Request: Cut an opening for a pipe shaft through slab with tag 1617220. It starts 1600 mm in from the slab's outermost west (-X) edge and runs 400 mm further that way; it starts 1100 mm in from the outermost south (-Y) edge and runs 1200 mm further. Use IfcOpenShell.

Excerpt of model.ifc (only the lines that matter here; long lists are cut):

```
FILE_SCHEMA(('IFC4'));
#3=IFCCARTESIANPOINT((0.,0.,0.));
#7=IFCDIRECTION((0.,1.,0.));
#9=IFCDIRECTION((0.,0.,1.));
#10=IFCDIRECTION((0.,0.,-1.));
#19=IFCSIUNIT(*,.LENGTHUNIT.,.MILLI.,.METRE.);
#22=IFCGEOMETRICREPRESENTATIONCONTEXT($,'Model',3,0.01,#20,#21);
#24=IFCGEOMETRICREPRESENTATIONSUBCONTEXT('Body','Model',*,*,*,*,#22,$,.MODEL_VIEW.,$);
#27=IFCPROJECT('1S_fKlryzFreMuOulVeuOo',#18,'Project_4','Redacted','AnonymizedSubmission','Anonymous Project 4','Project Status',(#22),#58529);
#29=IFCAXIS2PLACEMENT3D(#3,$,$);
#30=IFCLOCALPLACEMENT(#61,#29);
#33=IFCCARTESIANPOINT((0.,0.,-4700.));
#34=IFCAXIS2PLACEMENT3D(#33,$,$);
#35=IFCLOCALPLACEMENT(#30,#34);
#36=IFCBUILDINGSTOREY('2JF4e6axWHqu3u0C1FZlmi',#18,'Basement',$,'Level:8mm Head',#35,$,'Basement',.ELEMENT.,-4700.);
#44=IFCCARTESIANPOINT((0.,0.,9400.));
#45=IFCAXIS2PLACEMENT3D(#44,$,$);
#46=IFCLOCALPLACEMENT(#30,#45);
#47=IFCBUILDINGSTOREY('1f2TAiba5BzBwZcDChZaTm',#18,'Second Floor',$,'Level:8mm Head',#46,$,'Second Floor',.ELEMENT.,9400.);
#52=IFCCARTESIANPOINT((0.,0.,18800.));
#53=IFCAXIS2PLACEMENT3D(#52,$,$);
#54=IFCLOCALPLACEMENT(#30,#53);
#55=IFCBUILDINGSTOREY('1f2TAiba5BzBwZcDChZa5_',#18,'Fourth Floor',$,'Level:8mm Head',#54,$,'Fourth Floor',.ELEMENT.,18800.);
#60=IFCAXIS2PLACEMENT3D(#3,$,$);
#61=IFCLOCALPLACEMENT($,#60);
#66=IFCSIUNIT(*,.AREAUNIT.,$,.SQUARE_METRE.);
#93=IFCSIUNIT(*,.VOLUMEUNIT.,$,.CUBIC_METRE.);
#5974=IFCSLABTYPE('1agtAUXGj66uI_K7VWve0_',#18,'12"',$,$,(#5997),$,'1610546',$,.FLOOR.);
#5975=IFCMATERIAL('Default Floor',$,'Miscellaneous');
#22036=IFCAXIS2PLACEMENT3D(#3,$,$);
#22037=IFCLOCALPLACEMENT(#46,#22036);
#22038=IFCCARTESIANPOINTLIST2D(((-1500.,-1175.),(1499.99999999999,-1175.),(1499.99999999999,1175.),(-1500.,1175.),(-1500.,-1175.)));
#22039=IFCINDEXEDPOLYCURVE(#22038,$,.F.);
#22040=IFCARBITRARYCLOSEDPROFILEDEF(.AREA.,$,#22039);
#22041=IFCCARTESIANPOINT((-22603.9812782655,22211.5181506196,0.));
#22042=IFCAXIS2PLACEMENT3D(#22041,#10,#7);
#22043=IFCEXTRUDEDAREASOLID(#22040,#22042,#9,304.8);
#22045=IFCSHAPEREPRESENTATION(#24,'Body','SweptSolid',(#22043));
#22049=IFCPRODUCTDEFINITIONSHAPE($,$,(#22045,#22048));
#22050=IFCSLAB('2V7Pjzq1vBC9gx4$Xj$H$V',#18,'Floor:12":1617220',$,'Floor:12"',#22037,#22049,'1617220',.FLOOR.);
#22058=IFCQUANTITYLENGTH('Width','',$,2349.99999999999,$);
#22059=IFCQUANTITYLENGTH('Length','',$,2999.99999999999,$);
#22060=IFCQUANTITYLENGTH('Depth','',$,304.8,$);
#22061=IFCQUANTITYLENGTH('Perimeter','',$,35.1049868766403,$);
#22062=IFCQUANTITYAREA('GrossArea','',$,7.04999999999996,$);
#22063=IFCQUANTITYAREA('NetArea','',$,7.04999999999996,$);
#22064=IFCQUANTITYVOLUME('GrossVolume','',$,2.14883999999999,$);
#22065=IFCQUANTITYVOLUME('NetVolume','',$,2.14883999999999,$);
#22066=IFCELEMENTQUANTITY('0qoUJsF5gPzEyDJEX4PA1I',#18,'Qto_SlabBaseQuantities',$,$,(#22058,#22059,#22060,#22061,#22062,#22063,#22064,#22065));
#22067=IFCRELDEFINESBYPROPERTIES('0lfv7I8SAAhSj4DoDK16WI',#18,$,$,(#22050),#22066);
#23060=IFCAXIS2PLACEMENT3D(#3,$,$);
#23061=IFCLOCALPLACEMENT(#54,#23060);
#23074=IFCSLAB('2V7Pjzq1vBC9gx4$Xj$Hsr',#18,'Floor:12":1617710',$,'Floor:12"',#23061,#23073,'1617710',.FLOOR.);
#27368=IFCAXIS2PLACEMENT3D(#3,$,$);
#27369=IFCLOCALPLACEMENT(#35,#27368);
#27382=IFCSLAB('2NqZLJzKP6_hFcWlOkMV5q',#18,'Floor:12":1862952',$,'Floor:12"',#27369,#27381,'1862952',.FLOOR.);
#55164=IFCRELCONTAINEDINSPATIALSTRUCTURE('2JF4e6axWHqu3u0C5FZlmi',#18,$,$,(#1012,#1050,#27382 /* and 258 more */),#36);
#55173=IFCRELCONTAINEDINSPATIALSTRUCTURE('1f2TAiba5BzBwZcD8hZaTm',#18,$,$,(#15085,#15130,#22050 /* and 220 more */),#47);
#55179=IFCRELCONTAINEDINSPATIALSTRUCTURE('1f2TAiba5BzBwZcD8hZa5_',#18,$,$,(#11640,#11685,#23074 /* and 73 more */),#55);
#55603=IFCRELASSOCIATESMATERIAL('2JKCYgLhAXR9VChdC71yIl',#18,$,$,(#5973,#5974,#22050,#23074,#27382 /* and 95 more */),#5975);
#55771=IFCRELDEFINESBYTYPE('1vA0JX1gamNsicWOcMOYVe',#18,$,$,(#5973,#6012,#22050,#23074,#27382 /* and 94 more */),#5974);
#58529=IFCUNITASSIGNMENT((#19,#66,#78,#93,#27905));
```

```python
import numpy as np
import ifcopenshell
import ifcopenshell.api.feature
import ifcopenshell.api.geometry
import ifcopenshell.api.pset
import ifcopenshell.api.root
import ifcopenshell.geom
import ifcopenshell.util.element
import ifcopenshell.util.placement
import ifcopenshell.util.representation
import ifcopenshell.util.shape
import ifcopenshell.util.unit

model = ifcopenshell.open("model.ifc")
unit_scale = ifcopenshell.util.unit.calculate_unit_scale(model)
area_scale = ifcopenshell.util.unit.calculate_unit_scale(model, "AREAUNIT")
volume_scale = ifcopenshell.util.unit.calculate_unit_scale(model, "VOLUMEUNIT")
settings = ifcopenshell.geom.settings()


def volume(element):
    """Net volume in cubic metres, openings subtracted."""
    shape = ifcopenshell.geom.create_shape(settings, element)
    return ifcopenshell.util.shape.get_volume(shape.geometry)


slab = model.by_id(22050)
before = volume(slab)

# Extent in the slab's own axes, in metres. The edges named are its -X and -Y sides.
slab_shape = ifcopenshell.geom.create_shape(settings, slab)
vertices = ifcopenshell.util.shape.get_vertices(slab_shape.geometry)
x_min, y_min, bottom = vertices.min(axis=0)
top = vertices[:, 2].max()

opening = ifcopenshell.api.root.create_entity(model, ifc_class="IfcOpeningElement", name="Pipe shaft opening", predefined_type="OPENING")
context = ifcopenshell.util.representation.get_context(model, "Model", "Body", "MODEL_VIEW")
width, depth = 0.4, 1.2
outline = [(0.0, 0.0), (width, 0.0), (width, depth), (0.0, depth), (0.0, 0.0)]
# Overshoot both faces by 50 mm so the cut is clean.
shape = ifcopenshell.api.geometry.add_slab_representation(
    model, context=context, depth=top - bottom + 0.1, polyline=outline
)
ifcopenshell.api.geometry.assign_representation(model, product=opening, representation=shape)

matrix = ifcopenshell.util.placement.get_local_placement(slab.ObjectPlacement)
matrix[:, 3] = matrix @ np.append(np.array([x_min + 1.6, y_min + 1.1, bottom - 0.05]) / unit_scale, 1.0)
ifcopenshell.api.geometry.edit_object_placement(model, product=opening, matrix=matrix, is_si=False)
ifcopenshell.api.feature.add_feature(model, feature=opening, element=slab)

after = volume(slab)

# Update the slab's stored quantities.
qto = model.by_id(ifcopenshell.util.element.get_pset(slab, "Qto_SlabBaseQuantities", should_inherit=False)["id"])
ifcopenshell.api.pset.edit_qto(model, qto=qto, properties={
    "NetArea": after / (top - bottom) / area_scale,
    "NetVolume": after / volume_scale,
})

print(f"slab volume {before:.3f} -> {after:.3f} m3")

model.write("model_edited.ifc")
```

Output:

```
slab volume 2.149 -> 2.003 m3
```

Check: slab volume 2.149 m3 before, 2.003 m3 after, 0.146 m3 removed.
